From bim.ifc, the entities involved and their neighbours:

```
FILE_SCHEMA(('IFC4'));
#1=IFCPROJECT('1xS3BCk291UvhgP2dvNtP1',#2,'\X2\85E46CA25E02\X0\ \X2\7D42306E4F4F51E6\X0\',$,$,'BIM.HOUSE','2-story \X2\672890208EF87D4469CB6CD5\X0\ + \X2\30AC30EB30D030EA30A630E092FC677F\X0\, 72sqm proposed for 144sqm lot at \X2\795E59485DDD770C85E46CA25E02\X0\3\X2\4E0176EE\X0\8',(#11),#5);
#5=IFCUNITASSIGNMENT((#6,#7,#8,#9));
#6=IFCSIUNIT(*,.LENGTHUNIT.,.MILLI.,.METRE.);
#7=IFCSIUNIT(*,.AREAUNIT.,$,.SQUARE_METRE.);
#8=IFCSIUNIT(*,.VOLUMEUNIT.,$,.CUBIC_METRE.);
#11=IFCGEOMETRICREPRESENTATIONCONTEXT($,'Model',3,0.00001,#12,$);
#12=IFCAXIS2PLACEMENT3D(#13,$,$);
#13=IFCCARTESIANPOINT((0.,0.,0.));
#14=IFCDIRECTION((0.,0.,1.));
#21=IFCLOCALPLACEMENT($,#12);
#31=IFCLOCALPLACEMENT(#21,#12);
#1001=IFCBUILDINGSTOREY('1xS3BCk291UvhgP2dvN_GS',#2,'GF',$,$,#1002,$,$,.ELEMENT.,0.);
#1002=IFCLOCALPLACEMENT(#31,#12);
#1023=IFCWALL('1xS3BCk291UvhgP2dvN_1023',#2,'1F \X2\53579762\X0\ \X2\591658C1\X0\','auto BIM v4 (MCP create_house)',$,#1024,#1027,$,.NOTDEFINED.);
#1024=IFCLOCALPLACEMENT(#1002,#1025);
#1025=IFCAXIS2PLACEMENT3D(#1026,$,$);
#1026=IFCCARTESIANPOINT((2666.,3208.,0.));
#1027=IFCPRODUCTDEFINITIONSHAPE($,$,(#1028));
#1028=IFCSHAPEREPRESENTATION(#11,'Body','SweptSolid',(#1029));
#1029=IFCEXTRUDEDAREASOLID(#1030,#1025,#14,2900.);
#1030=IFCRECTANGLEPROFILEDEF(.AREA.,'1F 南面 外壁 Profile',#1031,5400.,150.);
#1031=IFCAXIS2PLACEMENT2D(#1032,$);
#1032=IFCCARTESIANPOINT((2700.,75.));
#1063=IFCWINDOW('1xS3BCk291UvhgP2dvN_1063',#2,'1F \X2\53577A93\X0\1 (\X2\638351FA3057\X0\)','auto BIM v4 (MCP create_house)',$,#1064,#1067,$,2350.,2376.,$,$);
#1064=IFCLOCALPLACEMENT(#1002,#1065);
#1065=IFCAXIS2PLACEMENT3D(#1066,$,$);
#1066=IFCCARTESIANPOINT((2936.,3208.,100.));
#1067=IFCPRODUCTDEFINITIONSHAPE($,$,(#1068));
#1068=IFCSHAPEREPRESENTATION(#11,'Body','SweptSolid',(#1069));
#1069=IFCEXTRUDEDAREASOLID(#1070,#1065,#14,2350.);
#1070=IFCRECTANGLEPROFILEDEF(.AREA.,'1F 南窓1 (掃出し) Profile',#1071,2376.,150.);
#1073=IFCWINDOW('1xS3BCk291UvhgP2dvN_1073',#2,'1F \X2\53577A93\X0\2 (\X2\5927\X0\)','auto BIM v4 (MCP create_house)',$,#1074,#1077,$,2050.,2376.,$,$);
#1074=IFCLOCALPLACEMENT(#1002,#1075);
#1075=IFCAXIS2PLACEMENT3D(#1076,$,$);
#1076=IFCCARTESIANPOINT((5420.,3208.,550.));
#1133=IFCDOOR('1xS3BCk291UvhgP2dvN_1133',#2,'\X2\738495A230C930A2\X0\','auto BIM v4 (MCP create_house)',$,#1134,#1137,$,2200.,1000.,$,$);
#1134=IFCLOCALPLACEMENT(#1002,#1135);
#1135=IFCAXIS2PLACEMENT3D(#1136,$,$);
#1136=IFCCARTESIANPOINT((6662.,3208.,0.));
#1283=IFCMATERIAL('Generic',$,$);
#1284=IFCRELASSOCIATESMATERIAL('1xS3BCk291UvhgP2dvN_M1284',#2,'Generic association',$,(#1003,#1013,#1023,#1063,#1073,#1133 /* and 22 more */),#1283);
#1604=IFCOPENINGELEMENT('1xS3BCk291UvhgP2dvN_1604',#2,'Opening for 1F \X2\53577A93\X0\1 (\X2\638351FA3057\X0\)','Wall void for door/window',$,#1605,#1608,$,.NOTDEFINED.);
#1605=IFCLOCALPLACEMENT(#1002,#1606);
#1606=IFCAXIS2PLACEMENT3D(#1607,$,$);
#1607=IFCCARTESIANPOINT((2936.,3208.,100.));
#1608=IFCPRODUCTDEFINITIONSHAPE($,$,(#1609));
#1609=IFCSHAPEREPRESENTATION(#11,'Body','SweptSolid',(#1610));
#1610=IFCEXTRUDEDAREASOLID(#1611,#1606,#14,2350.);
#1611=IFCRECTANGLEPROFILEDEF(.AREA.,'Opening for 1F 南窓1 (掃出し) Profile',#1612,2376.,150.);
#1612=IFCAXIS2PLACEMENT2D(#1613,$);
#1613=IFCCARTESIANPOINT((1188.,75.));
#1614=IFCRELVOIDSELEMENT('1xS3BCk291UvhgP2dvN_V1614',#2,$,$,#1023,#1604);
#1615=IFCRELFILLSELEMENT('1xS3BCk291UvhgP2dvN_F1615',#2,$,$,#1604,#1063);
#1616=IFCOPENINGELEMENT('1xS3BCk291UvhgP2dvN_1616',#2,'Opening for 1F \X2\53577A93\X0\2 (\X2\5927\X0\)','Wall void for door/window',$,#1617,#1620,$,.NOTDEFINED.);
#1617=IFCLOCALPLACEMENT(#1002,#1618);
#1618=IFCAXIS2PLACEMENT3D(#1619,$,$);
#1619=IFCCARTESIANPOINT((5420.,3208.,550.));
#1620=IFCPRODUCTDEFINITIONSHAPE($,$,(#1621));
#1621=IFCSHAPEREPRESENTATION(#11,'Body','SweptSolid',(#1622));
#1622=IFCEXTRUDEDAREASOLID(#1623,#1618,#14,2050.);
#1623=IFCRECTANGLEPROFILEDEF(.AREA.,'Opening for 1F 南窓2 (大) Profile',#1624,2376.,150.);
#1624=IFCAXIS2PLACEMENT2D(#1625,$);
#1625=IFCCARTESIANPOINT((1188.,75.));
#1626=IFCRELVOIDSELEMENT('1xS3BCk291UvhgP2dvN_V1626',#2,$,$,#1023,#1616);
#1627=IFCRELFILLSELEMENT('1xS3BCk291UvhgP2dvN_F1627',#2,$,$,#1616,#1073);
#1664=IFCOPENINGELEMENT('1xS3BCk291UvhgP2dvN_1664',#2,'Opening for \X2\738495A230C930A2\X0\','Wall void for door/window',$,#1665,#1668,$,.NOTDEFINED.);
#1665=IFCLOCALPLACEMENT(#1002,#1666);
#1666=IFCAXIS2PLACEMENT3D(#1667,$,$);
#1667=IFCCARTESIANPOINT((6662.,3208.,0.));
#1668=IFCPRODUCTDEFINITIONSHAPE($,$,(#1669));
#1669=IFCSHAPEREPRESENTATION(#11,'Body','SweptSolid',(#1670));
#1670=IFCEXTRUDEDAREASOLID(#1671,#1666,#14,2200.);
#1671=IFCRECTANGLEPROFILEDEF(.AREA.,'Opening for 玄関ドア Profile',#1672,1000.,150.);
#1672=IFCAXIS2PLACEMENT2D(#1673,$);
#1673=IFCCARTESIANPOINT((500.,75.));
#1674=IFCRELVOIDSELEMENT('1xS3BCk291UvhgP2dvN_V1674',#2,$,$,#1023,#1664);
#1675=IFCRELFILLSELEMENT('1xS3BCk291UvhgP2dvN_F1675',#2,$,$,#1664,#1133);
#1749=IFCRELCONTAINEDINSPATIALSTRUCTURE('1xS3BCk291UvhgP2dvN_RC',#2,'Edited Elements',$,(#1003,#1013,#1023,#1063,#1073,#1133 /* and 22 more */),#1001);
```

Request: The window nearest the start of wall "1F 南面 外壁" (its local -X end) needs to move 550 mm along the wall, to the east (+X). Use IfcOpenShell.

```python
import ifcopenshell
import ifcopenshell.api.geometry
import ifcopenshell.util.placement

model = ifcopenshell.open("bim.ifc")

window = model.by_guid("1xS3BCk291UvhgP2dvN_1063")
opening = window.FillsVoids[0].RelatingOpeningElement
wall = opening.VoidsElements[0].RelatingBuildingElement

wall_matrix = ifcopenshell.util.placement.get_local_placement(wall.ObjectPlacement)
shift = wall_matrix[:3, 0] * 550.0
before = ifcopenshell.util.placement.get_local_placement(window.ObjectPlacement)[:3, 3].copy()

# The window is not placed relative to its opening, so move both.
for product in (opening, window):
    matrix = ifcopenshell.util.placement.get_local_placement(product.ObjectPlacement)
    matrix[:3, 3] += shift
    ifcopenshell.api.geometry.edit_object_placement(model, product=product, matrix=matrix, is_si=False)

after = ifcopenshell.util.placement.get_local_placement(window.ObjectPlacement)[:3, 3]
print("window moved by", (after - before).round(3) + 0.0)

model.write("bim-out.ifc")
```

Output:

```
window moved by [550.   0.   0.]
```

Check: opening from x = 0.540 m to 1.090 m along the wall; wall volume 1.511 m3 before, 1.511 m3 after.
